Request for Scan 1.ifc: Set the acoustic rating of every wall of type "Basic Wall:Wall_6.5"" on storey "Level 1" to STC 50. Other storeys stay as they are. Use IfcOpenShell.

First a look at what the model holds.

```python
import ifcopenshell
import ifcopenshell.util.element

model = ifcopenshell.open("Scan 1.ifc")
print(model.schema)
storey = next(s for s in model.by_type("IfcBuildingStorey") if s.Name == "Level 1")
walls = [e for e in ifcopenshell.util.element.get_decomposition(storey) if e.is_a("IfcWall")]
seen = {}
for e in walls:
    element_type = ifcopenshell.util.element.get_type(e)
    key = (element_type.Name if element_type != e and element_type else None, ifcopenshell.util.element.get_pset(e, "Pset_WallCommon", "AcousticRating"))
    seen[key] = seen.get(key, 0) + 1
for (name, value), count in sorted(seen.items(), key=str):
    print(count, "x", name, "|", value)
```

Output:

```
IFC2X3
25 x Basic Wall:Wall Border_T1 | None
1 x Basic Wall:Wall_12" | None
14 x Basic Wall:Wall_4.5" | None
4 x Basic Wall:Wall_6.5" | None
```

```python
import ifcopenshell
import ifcopenshell.api.pset
import ifcopenshell.util.element

model = ifcopenshell.open("Scan 1.ifc")

storey = next(s for s in model.by_type("IfcBuildingStorey") if s.Name == "Level 1")
walls = [e for e in ifcopenshell.util.element.get_decomposition(storey) if e.is_a("IfcWall")]

count = 0
for e in walls:
    element_type = ifcopenshell.util.element.get_type(e)
    if element_type in (None, e) or element_type.Name != 'Basic Wall:Wall_6.5"':
        continue
    # add_pset returns the element's existing set when there is one.
    pset = ifcopenshell.api.pset.add_pset(model, product=e, name="Pset_WallCommon")
    ifcopenshell.api.pset.edit_pset(model, pset=pset, properties={"AcousticRating": "STC 50"})
    count += 1

print(count, "walls updated")

model.write("Scan 1_rev.ifc")
```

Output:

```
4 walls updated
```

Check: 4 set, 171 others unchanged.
